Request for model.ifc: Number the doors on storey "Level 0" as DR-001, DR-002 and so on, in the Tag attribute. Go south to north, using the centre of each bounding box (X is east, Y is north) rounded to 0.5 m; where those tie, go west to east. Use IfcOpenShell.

First a look at what the model holds.

```python
import ifcopenshell
import ifcopenshell.util.element
import ifcopenshell.util.placement

model = ifcopenshell.open("model.ifc")
print(model.schema)
storey = next(s for s in model.by_type("IfcBuildingStorey") if s.Name == "Level 0")
doors = [e for e in ifcopenshell.util.element.get_decomposition(storey) if e.is_a("IfcDoor")]
for e in sorted(doors, key=lambda e: e.id()):
    origin = ifcopenshell.util.placement.get_local_placement(e.ObjectPlacement)[:3, 3]
    print(e.id(), e.Tag, e.Name, origin.round(2) + 0.0, sep=" | ")
```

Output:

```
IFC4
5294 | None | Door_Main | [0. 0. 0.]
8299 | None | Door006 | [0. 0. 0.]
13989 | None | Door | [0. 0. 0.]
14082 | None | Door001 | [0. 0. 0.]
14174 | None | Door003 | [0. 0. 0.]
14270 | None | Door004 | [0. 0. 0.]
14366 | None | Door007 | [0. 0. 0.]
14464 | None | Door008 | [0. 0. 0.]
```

```python
import ifcopenshell
import ifcopenshell.geom
import ifcopenshell.util.element
import ifcopenshell.util.shape

model = ifcopenshell.open("model.ifc")
settings = ifcopenshell.geom.settings()
settings.set("use-world-coords", True)


def centre(element):
    shape = ifcopenshell.geom.create_shape(settings, element)
    return ifcopenshell.util.shape.get_bbox_centroid(shape.geometry)


storey = next(s for s in model.by_type("IfcBuildingStorey") if s.Name == "Level 0")
doors = [e for e in ifcopenshell.util.element.get_decomposition(storey) if e.is_a("IfcDoor")]

# Insertion points can sit at a corner or the storey origin, so sort by the geometry (in metres).
centres = {e: centre(e) for e in doors}
doors.sort(key=lambda e: (round(centres[e][1] / 0.5), centres[e][0]))

for i, e in enumerate(doors, start=1):
    number = f"DR-0{i:02d}"
    e.Tag = number
    print(e.id(), number)

model.write("model_edited.ifc")
```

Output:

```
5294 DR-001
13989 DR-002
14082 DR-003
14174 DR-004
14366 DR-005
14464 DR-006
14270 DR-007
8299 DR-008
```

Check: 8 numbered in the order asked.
